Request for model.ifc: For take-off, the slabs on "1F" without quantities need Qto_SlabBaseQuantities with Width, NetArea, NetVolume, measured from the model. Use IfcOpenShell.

First a look at what the model holds.

```python
import ifcopenshell
import ifcopenshell.util.element
import ifcopenshell.util.unit

model = ifcopenshell.open("model.ifc")
print(model.schema)
for unit_type in ("LENGTHUNIT", "AREAUNIT", "VOLUMEUNIT"):
    print(unit_type, ifcopenshell.util.unit.calculate_unit_scale(model, unit_type))
storey = next(s for s in model.by_type("IfcBuildingStorey") if s.Name == "1F")
slabs = [e for e in ifcopenshell.util.element.get_decomposition(storey) if e.is_a("IfcSlab")]
for e in sorted(slabs, key=lambda e: e.id()):
    print(e.id(), e.is_a(), e.Name, list(ifcopenshell.util.element.get_psets(e, qtos_only=True)), sep=" | ")
```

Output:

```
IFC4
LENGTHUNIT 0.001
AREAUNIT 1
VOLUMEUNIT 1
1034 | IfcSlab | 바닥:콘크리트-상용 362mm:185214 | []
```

```python
import ifcopenshell
import ifcopenshell.api.pset
import ifcopenshell.geom
import ifcopenshell.util.element
import ifcopenshell.util.shape
import ifcopenshell.util.unit

model = ifcopenshell.open("model.ifc")
unit_scale = ifcopenshell.util.unit.calculate_unit_scale(model)
area_scale = ifcopenshell.util.unit.calculate_unit_scale(model, "AREAUNIT")
volume_scale = ifcopenshell.util.unit.calculate_unit_scale(model, "VOLUMEUNIT")
settings = ifcopenshell.geom.settings()

storey = next(s for s in model.by_type("IfcBuildingStorey") if s.Name == "1F")
slabs = [e for e in ifcopenshell.util.element.get_decomposition(storey) if e.is_a("IfcSlab")]

for e in sorted(slabs, key=lambda e: e.id()):
    if ifcopenshell.util.element.get_psets(e, qtos_only=True, should_inherit=False):
        continue
    # Geometry comes back in metres, in the element's own axes.
    shape = ifcopenshell.geom.create_shape(settings, e)
    values = {
        "Width": ifcopenshell.util.shape.get_z(shape.geometry) / unit_scale,
        "NetArea": ifcopenshell.util.shape.get_footprint_area(shape.geometry) / area_scale,
        "NetVolume": ifcopenshell.util.shape.get_volume(shape.geometry) / volume_scale,
    }
    qto = ifcopenshell.api.pset.add_qto(model, product=e, name="Qto_SlabBaseQuantities")
    ifcopenshell.api.pset.edit_qto(model, qto=qto, properties=values)
    print(e.id(), {k: round(v, 3) for k, v in values.items()})

model.write("model-out.ifc")
```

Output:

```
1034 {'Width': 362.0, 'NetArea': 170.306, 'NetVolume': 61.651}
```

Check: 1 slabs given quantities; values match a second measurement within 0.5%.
